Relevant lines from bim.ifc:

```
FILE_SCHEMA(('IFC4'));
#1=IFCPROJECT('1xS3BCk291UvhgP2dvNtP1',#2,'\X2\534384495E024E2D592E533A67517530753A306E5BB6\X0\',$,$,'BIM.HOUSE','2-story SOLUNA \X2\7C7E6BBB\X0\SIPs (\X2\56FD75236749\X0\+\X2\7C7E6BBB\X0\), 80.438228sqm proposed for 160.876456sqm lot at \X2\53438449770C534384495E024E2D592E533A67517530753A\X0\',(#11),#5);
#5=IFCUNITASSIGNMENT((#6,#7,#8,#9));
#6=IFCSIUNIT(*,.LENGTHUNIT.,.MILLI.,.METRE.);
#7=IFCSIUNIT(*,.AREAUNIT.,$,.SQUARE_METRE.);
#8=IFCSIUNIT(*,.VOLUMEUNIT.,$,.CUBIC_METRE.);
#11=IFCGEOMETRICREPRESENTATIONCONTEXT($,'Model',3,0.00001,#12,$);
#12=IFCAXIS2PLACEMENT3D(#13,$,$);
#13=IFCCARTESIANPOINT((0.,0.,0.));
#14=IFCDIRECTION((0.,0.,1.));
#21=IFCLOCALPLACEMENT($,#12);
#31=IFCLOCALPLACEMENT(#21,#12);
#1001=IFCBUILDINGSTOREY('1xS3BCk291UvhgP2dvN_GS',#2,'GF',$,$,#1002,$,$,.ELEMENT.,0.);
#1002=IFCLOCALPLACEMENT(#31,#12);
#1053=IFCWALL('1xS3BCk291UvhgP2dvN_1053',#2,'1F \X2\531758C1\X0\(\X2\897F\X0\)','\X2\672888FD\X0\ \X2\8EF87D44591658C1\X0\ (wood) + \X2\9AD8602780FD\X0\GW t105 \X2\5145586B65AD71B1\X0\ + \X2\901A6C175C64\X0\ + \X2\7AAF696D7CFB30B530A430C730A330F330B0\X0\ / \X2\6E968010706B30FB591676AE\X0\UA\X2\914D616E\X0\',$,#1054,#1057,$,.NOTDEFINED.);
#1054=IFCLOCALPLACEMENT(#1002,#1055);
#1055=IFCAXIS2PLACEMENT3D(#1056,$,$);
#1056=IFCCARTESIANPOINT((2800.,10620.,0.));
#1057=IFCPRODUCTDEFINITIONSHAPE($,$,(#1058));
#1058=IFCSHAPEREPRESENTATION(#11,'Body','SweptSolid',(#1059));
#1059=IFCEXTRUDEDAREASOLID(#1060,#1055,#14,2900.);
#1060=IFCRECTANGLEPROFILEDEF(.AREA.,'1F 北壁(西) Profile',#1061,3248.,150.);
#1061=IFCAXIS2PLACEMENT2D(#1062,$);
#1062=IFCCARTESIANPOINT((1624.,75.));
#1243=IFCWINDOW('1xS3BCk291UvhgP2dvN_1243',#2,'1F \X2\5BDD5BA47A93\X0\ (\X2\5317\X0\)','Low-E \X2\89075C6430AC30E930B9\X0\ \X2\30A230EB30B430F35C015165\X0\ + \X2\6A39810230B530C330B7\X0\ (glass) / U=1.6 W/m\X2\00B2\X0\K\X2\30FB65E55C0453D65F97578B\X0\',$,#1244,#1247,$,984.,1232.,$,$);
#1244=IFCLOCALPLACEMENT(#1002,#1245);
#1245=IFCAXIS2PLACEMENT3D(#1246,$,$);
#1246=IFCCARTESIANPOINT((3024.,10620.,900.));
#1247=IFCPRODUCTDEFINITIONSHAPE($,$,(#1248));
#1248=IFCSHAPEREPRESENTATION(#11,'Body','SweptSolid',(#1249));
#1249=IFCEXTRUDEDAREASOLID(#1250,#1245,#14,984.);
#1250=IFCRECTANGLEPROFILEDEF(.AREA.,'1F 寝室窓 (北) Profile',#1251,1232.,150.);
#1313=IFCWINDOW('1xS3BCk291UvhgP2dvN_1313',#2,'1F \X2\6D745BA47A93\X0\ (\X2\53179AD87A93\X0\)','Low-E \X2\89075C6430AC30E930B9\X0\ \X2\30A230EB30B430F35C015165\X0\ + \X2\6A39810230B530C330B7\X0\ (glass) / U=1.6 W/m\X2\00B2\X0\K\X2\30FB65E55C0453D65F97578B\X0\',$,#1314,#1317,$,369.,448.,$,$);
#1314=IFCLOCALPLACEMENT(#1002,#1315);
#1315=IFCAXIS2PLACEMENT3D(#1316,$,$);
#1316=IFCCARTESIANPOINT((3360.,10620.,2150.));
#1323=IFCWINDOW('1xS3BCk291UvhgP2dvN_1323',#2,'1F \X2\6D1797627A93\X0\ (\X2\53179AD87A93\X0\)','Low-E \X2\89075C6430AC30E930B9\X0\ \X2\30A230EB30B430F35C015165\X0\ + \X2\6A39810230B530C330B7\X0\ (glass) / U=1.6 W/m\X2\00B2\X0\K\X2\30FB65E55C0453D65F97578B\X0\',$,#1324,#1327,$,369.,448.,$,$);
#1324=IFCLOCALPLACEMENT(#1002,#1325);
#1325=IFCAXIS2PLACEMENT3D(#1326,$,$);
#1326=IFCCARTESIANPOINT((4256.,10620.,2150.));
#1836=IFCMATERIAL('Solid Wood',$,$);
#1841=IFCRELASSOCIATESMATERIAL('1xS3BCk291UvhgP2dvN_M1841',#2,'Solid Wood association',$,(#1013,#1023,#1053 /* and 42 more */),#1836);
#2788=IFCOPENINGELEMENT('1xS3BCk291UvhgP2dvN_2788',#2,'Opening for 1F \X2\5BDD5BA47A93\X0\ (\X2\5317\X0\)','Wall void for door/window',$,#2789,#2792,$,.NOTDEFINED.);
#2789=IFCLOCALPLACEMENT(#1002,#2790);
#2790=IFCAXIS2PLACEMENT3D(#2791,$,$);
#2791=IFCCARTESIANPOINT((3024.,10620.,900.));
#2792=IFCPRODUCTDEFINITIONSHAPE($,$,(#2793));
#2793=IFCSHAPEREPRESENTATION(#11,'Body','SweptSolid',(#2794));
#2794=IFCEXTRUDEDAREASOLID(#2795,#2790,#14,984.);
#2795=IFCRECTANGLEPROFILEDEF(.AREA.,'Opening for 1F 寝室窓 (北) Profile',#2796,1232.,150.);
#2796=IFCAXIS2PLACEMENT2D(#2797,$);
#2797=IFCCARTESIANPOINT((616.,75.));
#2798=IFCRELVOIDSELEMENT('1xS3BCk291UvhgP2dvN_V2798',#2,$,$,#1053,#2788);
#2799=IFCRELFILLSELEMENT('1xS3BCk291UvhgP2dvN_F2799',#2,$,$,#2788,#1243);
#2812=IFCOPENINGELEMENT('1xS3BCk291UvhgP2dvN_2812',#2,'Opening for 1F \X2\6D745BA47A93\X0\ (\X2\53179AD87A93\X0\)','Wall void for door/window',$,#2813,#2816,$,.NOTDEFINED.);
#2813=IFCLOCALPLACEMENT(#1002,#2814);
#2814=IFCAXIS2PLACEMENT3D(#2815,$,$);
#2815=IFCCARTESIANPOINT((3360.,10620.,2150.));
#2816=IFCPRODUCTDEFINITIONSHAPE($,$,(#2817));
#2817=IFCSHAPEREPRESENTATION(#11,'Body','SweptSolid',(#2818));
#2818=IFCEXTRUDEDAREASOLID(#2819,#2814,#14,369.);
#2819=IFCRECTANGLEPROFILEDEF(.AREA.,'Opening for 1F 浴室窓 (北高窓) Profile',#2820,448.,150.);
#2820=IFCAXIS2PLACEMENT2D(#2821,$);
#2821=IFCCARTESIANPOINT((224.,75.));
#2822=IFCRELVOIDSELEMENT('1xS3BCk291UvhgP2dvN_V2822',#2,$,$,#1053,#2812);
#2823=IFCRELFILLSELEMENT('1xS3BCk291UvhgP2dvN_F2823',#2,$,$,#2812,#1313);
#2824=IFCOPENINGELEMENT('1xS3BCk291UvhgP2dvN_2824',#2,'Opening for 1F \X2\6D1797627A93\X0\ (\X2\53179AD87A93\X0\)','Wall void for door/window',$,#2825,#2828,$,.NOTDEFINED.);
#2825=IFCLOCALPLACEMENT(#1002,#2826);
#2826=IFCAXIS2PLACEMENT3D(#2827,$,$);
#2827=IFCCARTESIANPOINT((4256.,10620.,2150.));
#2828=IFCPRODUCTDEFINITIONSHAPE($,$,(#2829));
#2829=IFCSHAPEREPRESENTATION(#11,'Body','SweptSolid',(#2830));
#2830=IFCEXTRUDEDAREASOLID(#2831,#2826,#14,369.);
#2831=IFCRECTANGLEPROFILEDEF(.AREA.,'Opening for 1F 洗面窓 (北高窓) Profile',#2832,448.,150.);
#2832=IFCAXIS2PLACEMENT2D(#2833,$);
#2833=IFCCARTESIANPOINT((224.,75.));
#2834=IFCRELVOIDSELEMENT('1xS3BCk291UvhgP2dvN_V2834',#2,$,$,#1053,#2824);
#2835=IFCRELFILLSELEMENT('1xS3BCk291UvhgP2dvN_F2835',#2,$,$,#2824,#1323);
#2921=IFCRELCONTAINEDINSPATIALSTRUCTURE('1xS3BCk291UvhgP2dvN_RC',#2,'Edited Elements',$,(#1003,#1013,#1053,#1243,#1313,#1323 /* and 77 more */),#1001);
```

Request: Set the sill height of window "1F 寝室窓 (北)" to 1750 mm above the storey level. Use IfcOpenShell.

```python
import numpy as np
import ifcopenshell
import ifcopenshell.api.geometry
import ifcopenshell.geom
import ifcopenshell.util.element
import ifcopenshell.util.placement
import ifcopenshell.util.shape
import ifcopenshell.util.unit

model = ifcopenshell.open("bim.ifc")
unit_scale = ifcopenshell.util.unit.calculate_unit_scale(model)

window = model.by_guid("1xS3BCk291UvhgP2dvN_1243")
opening = window.FillsVoids[0].RelatingOpeningElement
storey = ifcopenshell.util.element.get_container(window, ifc_class="IfcBuildingStorey")
level = ifcopenshell.util.placement.get_local_placement(storey.ObjectPlacement)[2, 3]

# The opening's origin need not be at the sill, so measure its lowest point.
shape = ifcopenshell.geom.create_shape(ifcopenshell.geom.settings(), opening)
bottom = ifcopenshell.util.shape.get_shape_bottom_elevation(shape, shape.geometry) / unit_scale
dz = level + 1750.0 - bottom

shift = np.array([0.0, 0.0, dz])
# The window is not placed relative to its opening, so move both.
for product in (opening, window):
    matrix = ifcopenshell.util.placement.get_local_placement(product.ObjectPlacement)
    matrix[:3, 3] += shift
    ifcopenshell.api.geometry.edit_object_placement(model, product=product, matrix=matrix, is_si=False)

print(f"moved by {dz * unit_scale:+.3f} m")

model.write("bim_rev.ifc")
```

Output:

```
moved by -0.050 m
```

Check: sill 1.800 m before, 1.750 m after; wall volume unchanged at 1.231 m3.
